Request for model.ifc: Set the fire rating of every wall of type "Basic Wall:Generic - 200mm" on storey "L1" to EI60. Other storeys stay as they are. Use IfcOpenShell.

First a look at what the model holds.

```python
import ifcopenshell
import ifcopenshell.util.element

model = ifcopenshell.open("model.ifc")
print(model.schema)
storey = next(s for s in model.by_type("IfcBuildingStorey") if s.Name == "L1")
walls = [e for e in ifcopenshell.util.element.get_decomposition(storey) if e.is_a("IfcWall")]
seen = {}
for e in walls:
    element_type = ifcopenshell.util.element.get_type(e)
    key = (element_type.Name if element_type != e and element_type else None, ifcopenshell.util.element.get_pset(e, "Pset_WallCommon", "FireRating"))
    seen[key] = seen.get(key, 0) + 1
for (name, value), count in sorted(seen.items(), key=str):
    print(count, "x", name, "|", value)
```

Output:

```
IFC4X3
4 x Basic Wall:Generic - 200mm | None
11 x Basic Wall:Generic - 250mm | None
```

```python
import ifcopenshell
import ifcopenshell.api.pset
import ifcopenshell.util.element

model = ifcopenshell.open("model.ifc")

storey = next(s for s in model.by_type("IfcBuildingStorey") if s.Name == "L1")
walls = [e for e in ifcopenshell.util.element.get_decomposition(storey) if e.is_a("IfcWall")]

count = 0
for e in walls:
    element_type = ifcopenshell.util.element.get_type(e)
    if element_type in (None, e) or element_type.Name != "Basic Wall:Generic - 200mm":
        continue
    # add_pset returns the element's existing set when there is one.
    pset = ifcopenshell.api.pset.add_pset(model, product=e, name="Pset_WallCommon")
    ifcopenshell.api.pset.edit_pset(model, pset=pset, properties={"FireRating": "EI60"})
    count += 1

print(count, "walls updated")

model.write("model_v2.ifc")
```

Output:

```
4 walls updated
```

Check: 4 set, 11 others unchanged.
